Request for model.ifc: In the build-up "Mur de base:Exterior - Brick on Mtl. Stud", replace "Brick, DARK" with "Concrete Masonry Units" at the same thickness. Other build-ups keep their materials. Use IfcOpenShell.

First a look at what the model holds.

```python
import ifcopenshell
import ifcopenshell.util.element

model = ifcopenshell.open("model.ifc")
print(model.schema)
for layer_set in model.by_type("IfcMaterialLayerSet"):
    if layer_set.LayerSetName == "Mur de base:Exterior - Brick on Mtl. Stud":
        for layer in layer_set.MaterialLayers:
            print(layer.id(), layer.Material and layer.Material.Name, layer.LayerThickness, sep=" | ")
        print(len(ifcopenshell.util.element.get_elements_by_material(model, layer_set)), "elements and types use it")
print(sorted(m.Name for m in model.by_type("IfcMaterial") if m.Name)[:60])
```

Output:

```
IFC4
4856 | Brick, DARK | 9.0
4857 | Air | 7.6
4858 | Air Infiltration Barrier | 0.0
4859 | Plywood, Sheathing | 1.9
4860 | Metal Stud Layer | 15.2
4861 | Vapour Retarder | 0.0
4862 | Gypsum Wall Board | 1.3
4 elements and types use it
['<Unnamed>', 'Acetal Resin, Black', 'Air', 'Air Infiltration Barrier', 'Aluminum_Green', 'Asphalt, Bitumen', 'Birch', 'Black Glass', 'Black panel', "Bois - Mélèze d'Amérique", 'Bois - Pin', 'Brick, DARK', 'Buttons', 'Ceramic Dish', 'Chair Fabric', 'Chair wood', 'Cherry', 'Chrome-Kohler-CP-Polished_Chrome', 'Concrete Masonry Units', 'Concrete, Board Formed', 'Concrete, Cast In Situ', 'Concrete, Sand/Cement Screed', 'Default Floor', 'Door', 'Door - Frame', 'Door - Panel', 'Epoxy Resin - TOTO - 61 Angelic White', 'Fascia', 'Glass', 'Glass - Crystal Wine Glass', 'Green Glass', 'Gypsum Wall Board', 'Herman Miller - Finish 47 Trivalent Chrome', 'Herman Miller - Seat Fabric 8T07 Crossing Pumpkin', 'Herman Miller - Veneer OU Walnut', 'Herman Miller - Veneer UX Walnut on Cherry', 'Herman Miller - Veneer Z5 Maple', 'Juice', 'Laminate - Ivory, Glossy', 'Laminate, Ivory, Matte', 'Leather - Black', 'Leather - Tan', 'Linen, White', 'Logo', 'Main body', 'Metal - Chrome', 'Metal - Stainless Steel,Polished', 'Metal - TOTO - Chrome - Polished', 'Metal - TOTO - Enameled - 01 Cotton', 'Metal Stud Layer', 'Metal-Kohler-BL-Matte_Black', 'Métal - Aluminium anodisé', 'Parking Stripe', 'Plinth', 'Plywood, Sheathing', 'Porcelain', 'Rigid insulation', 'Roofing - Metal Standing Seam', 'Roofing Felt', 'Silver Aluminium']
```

```python
import ifcopenshell
import ifcopenshell.api.material

model = ifcopenshell.open("model.ifc")

layer_set = next(s for s in model.by_type("IfcMaterialLayerSet") if s.LayerSetName == "Mur de base:Exterior - Brick on Mtl. Stud")
layer = next(l for l in layer_set.MaterialLayers if l.Material and l.Material.Name == "Brick, DARK")
material = next(m for m in model.by_type("IfcMaterial") if m.Name == "Concrete Masonry Units")

# Point this one layer at the other material; renaming the old one would change it everywhere.
ifcopenshell.api.material.edit_layer(model, layer=layer, attributes={"Name": material.Name}, material=material)

print([l.Material.Name if l.Material else None for l in layer_set.MaterialLayers])

model.write("model-out.ifc")
```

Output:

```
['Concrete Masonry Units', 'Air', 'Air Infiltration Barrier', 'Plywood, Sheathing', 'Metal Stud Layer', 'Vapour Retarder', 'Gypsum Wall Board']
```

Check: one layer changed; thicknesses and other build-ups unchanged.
